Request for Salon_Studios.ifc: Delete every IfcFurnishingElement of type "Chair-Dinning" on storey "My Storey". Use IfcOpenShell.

First a look at what the model holds.

```python
import ifcopenshell
import ifcopenshell.util.element

model = ifcopenshell.open("Salon_Studios.ifc")
print(model.schema)
storey = next(s for s in model.by_type("IfcBuildingStorey") if s.Name == "My Storey")
furniture = [e for e in ifcopenshell.util.element.get_decomposition(storey) if e.is_a("IfcFurnishingElement")]
seen = {}
for e in furniture:
    element_type = ifcopenshell.util.element.get_type(e)
    name = element_type.Name if element_type not in (None, e) else None
    seen[name] = seen.get(name, 0) + 1
for name, count in sorted(seen.items(), key=str):
    print(count, "x", name)
```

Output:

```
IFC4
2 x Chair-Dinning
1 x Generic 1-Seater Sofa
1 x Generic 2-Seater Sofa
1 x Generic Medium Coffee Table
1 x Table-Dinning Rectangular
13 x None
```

```python
import ifcopenshell
import ifcopenshell.api.root
import ifcopenshell.util.element

model = ifcopenshell.open("Salon_Studios.ifc")

storey = next(s for s in model.by_type("IfcBuildingStorey") if s.Name == "My Storey")
furniture = [e for e in ifcopenshell.util.element.get_decomposition(storey) if e.is_a("IfcFurnishingElement")]
targets = [e for e in furniture if (t := ifcopenshell.util.element.get_type(e)) not in (None, e) and t.Name == "Chair-Dinning"]

for e in targets:
    ifcopenshell.api.root.remove_product(model, product=e)
print(len(targets), "removed")

model.write("Salon_Studios_rev.ifc")
```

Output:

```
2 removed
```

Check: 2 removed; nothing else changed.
